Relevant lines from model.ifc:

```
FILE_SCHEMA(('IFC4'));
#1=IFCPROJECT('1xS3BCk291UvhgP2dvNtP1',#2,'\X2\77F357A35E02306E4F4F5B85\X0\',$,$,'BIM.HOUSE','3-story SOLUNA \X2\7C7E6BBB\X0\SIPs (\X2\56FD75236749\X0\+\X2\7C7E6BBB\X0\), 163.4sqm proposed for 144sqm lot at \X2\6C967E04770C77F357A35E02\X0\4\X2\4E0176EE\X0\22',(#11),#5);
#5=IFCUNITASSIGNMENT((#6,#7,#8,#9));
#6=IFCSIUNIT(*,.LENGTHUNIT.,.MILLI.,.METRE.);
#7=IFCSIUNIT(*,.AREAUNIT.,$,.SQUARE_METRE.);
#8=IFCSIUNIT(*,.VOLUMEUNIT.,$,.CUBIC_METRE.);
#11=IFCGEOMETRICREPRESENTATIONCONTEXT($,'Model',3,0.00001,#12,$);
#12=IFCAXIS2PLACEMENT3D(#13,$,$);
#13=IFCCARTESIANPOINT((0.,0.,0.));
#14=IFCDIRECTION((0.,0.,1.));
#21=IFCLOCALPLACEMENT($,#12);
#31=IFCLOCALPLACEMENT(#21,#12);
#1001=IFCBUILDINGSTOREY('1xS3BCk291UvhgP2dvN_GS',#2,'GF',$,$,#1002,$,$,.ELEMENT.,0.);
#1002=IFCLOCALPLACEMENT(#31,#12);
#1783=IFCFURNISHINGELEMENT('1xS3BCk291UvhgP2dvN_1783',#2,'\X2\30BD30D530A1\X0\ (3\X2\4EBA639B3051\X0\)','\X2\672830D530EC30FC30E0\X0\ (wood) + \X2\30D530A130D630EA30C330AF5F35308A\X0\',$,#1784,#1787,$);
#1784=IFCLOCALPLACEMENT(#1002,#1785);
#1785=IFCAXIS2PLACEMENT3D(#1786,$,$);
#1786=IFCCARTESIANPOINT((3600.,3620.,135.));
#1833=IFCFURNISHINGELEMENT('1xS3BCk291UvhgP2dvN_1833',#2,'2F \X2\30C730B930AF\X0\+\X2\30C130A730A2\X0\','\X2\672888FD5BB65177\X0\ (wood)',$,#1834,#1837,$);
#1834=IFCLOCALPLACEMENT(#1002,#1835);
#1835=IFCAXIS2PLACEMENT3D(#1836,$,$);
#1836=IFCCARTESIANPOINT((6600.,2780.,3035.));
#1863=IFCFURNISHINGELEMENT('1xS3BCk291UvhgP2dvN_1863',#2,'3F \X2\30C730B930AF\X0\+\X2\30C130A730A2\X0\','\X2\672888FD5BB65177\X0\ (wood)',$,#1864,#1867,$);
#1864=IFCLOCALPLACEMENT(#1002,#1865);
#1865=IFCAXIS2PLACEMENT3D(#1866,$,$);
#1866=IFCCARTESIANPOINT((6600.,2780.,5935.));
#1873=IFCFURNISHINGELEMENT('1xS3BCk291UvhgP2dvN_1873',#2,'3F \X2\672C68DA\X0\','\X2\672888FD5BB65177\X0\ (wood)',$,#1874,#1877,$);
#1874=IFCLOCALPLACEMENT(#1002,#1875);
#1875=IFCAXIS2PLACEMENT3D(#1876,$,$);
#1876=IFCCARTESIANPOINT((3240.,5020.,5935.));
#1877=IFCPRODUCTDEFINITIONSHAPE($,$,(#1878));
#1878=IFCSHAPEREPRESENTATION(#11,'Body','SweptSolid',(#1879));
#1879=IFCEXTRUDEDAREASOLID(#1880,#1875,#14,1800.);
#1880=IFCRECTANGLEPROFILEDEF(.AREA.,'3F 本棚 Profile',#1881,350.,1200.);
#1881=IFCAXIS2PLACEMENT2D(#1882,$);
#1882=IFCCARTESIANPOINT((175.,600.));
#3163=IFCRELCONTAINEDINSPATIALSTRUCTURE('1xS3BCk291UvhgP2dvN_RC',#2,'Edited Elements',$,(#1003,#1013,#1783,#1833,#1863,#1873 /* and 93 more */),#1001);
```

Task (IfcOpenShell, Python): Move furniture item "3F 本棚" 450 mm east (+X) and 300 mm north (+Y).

```python
import ifcopenshell
import ifcopenshell.api.geometry
import ifcopenshell.util.placement

model = ifcopenshell.open("model.ifc")

item = model.by_guid("1xS3BCk291UvhgP2dvN_1873")
matrix = ifcopenshell.util.placement.get_local_placement(item.ObjectPlacement)
matrix[0, 3] += 450.0
matrix[1, 3] += 300.0
ifcopenshell.api.geometry.edit_object_placement(model, product=item, matrix=matrix, is_si=False)

print(ifcopenshell.util.placement.get_local_placement(item.ObjectPlacement).round(3) + 0.0)

model.write("model_rev.ifc")
```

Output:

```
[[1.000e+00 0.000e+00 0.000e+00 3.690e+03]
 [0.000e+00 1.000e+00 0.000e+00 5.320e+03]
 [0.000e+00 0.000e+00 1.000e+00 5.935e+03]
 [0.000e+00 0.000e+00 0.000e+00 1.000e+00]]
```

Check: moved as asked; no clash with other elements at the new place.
